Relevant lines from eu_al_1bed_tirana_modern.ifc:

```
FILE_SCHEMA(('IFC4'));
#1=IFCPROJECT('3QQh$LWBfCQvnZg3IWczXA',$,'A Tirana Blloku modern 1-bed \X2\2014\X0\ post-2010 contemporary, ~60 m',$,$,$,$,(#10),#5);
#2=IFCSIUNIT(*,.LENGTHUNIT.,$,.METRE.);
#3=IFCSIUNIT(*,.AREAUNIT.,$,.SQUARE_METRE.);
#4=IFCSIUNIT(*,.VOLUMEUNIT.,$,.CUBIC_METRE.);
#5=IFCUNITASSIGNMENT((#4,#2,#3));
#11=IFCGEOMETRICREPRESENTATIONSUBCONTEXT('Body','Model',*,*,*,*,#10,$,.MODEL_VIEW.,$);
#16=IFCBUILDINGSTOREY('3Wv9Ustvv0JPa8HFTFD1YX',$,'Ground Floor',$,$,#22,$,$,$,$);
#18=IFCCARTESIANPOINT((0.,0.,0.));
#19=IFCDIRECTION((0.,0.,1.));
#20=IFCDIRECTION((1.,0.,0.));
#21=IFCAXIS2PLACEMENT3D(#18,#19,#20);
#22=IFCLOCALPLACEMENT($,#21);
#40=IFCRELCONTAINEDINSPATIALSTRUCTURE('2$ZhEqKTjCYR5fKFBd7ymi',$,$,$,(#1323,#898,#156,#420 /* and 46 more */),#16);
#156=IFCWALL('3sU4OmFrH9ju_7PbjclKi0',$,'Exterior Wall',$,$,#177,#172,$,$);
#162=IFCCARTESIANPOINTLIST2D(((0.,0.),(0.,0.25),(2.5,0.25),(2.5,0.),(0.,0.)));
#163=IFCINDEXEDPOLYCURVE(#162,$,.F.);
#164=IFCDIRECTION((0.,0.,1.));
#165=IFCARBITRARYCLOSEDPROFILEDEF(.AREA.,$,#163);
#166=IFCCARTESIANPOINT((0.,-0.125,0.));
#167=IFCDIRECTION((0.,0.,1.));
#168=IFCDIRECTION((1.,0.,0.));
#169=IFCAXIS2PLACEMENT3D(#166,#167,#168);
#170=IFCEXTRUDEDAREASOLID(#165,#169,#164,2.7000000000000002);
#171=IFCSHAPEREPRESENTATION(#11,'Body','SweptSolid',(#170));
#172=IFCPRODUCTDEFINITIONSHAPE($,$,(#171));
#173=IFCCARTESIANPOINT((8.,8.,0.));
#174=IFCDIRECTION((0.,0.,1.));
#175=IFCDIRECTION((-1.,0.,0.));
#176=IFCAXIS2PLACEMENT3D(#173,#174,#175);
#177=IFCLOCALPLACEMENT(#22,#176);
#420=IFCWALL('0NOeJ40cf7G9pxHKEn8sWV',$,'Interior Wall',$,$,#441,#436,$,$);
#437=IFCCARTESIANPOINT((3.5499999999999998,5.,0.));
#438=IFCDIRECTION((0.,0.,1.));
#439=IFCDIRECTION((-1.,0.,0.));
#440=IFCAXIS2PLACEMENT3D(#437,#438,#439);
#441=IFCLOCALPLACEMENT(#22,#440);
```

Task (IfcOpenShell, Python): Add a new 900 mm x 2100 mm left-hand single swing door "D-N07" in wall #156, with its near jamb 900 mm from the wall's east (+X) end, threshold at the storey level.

```python
import numpy as np
import ifcopenshell
import ifcopenshell.api.feature
import ifcopenshell.api.geometry
import ifcopenshell.api.root
import ifcopenshell.api.spatial
import ifcopenshell.geom
import ifcopenshell.util.element
import ifcopenshell.util.placement
import ifcopenshell.util.representation
import ifcopenshell.util.shape
import ifcopenshell.util.unit

model = ifcopenshell.open("eu_al_1bed_tirana_modern.ifc")
unit_scale = ifcopenshell.util.unit.calculate_unit_scale(model)
settings = ifcopenshell.geom.settings()


def volume(element):
    """Net volume in cubic metres, openings subtracted."""
    shape = ifcopenshell.geom.create_shape(settings, element)
    return ifcopenshell.util.shape.get_volume(shape.geometry)


wall = model.by_id(156)
storey = ifcopenshell.util.element.get_container(wall, ifc_class="IfcBuildingStorey")
context = ifcopenshell.util.representation.get_context(model, "Model", "Body", "MODEL_VIEW")
before = volume(wall)

width, height, from_end, sill = 0.9, 2.1, 0.9, 0.0  # metres

# The wall runs along its own X axis, and the end named is its -X end.
wall_shape = ifcopenshell.geom.create_shape(settings, wall)
x, y, z = ifcopenshell.util.shape.get_vertices(wall_shape.geometry).T
start = x.min() + from_end
face, thickness = float(y.min()), float(y.max() - y.min())
wall_matrix = ifcopenshell.util.placement.get_local_placement(wall.ObjectPlacement)
level = ifcopenshell.util.placement.get_local_placement(storey.ObjectPlacement)[2, 3]


def in_wall(x, y):
    """Placement at x, y metres in the wall's axes, at sill height."""
    matrix = wall_matrix.copy()
    matrix[:, 3] = wall_matrix @ np.array([x / unit_scale, y / unit_scale, 0.0, 1.0])
    matrix[2, 3] = level + sill / unit_scale
    return matrix


# Opening: a box that overshoots both wall faces by 50 mm.
opening = ifcopenshell.api.root.create_entity(model, ifc_class="IfcOpeningElement", predefined_type="OPENING")
box = ifcopenshell.api.geometry.add_wall_representation(
    model, context=context, length=width, height=height, thickness=thickness + 0.1
)
ifcopenshell.api.geometry.assign_representation(model, product=opening, representation=box)
ifcopenshell.api.geometry.edit_object_placement(model, product=opening, matrix=in_wall(start, face - 0.05), is_si=False)
ifcopenshell.api.feature.add_feature(model, feature=opening, element=wall)

door = ifcopenshell.api.root.create_entity(model, ifc_class="IfcDoor", name="D-N07", predefined_type="DOOR")
door.OverallWidth, door.OverallHeight = width / unit_scale, height / unit_scale
door.OperationType = "SINGLE_SWING_LEFT"
body = ifcopenshell.api.geometry.add_door_representation(
    model,
    context=context,
    overall_width=door.OverallWidth,
    overall_height=door.OverallHeight,
    operation_type="SINGLE_SWING_LEFT",
    lining_properties={"LiningDepth": thickness / unit_scale, "ThresholdDepth": thickness / unit_scale},
)
ifcopenshell.api.geometry.assign_representation(model, product=door, representation=body)
ifcopenshell.api.spatial.assign_container(model, products=[door], relating_structure=storey)
ifcopenshell.api.feature.add_filling(model, opening=opening, element=door)

# The lining spans the wall, so the door starts at the wall face.
ifcopenshell.api.geometry.edit_object_placement(model, product=door, matrix=in_wall(start, face), is_si=False)

after = volume(wall)

print(f"wall volume {before:.3f} -> {after:.3f} m3")

model.write("eu_al_1bed_tirana_modern_edited.ifc")
```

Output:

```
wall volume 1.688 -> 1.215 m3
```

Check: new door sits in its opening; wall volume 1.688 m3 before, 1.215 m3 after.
